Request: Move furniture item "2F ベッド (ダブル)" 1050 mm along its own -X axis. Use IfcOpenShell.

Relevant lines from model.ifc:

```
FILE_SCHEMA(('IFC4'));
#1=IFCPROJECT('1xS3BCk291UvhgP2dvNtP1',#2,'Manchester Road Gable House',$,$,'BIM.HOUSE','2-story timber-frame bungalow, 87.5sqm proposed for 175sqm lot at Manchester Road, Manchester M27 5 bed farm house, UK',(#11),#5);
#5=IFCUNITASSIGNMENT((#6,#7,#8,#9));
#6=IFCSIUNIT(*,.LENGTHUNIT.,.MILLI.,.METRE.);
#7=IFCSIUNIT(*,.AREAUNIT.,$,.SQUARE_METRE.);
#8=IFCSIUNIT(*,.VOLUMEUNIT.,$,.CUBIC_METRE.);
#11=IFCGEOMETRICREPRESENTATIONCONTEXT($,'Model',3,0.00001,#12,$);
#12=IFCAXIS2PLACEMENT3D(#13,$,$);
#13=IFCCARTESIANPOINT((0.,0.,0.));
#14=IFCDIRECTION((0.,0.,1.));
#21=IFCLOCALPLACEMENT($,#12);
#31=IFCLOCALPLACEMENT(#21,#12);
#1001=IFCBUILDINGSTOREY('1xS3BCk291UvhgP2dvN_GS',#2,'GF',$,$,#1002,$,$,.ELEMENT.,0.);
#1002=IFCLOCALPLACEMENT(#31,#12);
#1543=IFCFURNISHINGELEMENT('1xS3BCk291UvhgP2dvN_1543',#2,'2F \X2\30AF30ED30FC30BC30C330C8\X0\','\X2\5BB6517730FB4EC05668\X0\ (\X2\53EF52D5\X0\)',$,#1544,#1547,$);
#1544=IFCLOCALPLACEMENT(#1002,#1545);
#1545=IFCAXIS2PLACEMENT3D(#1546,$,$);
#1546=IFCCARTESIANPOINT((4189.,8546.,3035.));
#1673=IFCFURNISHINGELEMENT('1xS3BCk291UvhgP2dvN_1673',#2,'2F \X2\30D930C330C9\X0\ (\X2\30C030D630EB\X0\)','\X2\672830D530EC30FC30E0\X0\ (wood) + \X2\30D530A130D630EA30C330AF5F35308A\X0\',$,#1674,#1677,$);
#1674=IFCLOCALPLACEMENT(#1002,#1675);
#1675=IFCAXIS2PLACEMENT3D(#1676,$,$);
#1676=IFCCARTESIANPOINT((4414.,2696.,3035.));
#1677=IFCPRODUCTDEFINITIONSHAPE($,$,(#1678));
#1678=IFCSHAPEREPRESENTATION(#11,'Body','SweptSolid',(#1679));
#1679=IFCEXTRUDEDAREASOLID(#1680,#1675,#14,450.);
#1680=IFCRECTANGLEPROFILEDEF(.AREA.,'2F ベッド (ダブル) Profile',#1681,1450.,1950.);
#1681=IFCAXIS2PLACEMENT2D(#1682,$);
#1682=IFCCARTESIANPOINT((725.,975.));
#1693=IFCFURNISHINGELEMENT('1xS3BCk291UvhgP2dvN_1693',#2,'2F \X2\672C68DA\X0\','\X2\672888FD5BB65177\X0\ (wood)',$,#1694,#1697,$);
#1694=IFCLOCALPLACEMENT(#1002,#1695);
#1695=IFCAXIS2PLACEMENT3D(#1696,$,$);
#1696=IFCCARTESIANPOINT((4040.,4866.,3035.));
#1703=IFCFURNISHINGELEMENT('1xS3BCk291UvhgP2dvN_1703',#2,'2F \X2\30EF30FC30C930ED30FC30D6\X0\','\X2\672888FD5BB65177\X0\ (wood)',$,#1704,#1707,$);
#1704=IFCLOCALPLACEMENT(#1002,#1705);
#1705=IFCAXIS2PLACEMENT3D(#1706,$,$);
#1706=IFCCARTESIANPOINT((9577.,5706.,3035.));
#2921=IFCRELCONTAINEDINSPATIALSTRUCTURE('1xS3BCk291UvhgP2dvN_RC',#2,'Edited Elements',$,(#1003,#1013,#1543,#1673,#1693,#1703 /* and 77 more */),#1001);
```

```python
import ifcopenshell
import ifcopenshell.api.geometry
import ifcopenshell.util.placement
import ifcopenshell.util.unit

model = ifcopenshell.open("model.ifc")
unit_scale = ifcopenshell.util.unit.calculate_unit_scale(model)

item = model.by_guid("1xS3BCk291UvhgP2dvN_1673")
matrix = ifcopenshell.util.placement.get_local_placement(item.ObjectPlacement)
matrix[:3, 3] -= matrix[:3, 0] * 1.05 / unit_scale
ifcopenshell.api.geometry.edit_object_placement(model, product=item, matrix=matrix, is_si=False)

print(ifcopenshell.util.placement.get_local_placement(item.ObjectPlacement).round(3) + 0.0)

model.write("model_rev.ifc")
```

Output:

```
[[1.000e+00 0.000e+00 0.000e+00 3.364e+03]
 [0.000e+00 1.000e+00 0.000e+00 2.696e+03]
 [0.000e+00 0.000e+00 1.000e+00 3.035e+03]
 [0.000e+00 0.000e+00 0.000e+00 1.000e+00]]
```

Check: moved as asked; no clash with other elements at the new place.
